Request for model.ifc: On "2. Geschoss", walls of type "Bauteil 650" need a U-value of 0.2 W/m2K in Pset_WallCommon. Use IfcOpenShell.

First a look at what the model holds.

```python
import ifcopenshell
import ifcopenshell.util.element

model = ifcopenshell.open("model.ifc")
print(model.schema)
storey = next(s for s in model.by_type("IfcBuildingStorey") if s.Name == "2. Geschoss")
walls = [e for e in ifcopenshell.util.element.get_decomposition(storey) if e.is_a("IfcWall")]
seen = {}
for e in walls:
    element_type = ifcopenshell.util.element.get_type(e)
    key = (element_type.Name if element_type != e and element_type else None, ifcopenshell.util.element.get_pset(e, "Pset_WallCommon", "ThermalTransmittance"))
    seen[key] = seen.get(key, 0) + 1
for (name, value), count in sorted(seen.items(), key=str):
    print(count, "x", name, "|", value)
```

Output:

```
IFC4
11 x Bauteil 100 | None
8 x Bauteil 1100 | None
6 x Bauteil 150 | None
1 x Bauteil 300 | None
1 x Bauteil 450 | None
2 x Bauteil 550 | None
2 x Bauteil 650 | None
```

```python
import ifcopenshell
import ifcopenshell.api.pset
import ifcopenshell.util.element

model = ifcopenshell.open("model.ifc")

storey = next(s for s in model.by_type("IfcBuildingStorey") if s.Name == "2. Geschoss")
walls = [e for e in ifcopenshell.util.element.get_decomposition(storey) if e.is_a("IfcWall")]

count = 0
for e in walls:
    element_type = ifcopenshell.util.element.get_type(e)
    if element_type in (None, e) or element_type.Name != "Bauteil 650":
        continue
    # add_pset returns the element's existing set when there is one.
    pset = ifcopenshell.api.pset.add_pset(model, product=e, name="Pset_WallCommon")
    ifcopenshell.api.pset.edit_pset(model, pset=pset, properties={"ThermalTransmittance": 0.2})
    count += 1

print(count, "walls updated")

model.write("model_v2.ifc")
```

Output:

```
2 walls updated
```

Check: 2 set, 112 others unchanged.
